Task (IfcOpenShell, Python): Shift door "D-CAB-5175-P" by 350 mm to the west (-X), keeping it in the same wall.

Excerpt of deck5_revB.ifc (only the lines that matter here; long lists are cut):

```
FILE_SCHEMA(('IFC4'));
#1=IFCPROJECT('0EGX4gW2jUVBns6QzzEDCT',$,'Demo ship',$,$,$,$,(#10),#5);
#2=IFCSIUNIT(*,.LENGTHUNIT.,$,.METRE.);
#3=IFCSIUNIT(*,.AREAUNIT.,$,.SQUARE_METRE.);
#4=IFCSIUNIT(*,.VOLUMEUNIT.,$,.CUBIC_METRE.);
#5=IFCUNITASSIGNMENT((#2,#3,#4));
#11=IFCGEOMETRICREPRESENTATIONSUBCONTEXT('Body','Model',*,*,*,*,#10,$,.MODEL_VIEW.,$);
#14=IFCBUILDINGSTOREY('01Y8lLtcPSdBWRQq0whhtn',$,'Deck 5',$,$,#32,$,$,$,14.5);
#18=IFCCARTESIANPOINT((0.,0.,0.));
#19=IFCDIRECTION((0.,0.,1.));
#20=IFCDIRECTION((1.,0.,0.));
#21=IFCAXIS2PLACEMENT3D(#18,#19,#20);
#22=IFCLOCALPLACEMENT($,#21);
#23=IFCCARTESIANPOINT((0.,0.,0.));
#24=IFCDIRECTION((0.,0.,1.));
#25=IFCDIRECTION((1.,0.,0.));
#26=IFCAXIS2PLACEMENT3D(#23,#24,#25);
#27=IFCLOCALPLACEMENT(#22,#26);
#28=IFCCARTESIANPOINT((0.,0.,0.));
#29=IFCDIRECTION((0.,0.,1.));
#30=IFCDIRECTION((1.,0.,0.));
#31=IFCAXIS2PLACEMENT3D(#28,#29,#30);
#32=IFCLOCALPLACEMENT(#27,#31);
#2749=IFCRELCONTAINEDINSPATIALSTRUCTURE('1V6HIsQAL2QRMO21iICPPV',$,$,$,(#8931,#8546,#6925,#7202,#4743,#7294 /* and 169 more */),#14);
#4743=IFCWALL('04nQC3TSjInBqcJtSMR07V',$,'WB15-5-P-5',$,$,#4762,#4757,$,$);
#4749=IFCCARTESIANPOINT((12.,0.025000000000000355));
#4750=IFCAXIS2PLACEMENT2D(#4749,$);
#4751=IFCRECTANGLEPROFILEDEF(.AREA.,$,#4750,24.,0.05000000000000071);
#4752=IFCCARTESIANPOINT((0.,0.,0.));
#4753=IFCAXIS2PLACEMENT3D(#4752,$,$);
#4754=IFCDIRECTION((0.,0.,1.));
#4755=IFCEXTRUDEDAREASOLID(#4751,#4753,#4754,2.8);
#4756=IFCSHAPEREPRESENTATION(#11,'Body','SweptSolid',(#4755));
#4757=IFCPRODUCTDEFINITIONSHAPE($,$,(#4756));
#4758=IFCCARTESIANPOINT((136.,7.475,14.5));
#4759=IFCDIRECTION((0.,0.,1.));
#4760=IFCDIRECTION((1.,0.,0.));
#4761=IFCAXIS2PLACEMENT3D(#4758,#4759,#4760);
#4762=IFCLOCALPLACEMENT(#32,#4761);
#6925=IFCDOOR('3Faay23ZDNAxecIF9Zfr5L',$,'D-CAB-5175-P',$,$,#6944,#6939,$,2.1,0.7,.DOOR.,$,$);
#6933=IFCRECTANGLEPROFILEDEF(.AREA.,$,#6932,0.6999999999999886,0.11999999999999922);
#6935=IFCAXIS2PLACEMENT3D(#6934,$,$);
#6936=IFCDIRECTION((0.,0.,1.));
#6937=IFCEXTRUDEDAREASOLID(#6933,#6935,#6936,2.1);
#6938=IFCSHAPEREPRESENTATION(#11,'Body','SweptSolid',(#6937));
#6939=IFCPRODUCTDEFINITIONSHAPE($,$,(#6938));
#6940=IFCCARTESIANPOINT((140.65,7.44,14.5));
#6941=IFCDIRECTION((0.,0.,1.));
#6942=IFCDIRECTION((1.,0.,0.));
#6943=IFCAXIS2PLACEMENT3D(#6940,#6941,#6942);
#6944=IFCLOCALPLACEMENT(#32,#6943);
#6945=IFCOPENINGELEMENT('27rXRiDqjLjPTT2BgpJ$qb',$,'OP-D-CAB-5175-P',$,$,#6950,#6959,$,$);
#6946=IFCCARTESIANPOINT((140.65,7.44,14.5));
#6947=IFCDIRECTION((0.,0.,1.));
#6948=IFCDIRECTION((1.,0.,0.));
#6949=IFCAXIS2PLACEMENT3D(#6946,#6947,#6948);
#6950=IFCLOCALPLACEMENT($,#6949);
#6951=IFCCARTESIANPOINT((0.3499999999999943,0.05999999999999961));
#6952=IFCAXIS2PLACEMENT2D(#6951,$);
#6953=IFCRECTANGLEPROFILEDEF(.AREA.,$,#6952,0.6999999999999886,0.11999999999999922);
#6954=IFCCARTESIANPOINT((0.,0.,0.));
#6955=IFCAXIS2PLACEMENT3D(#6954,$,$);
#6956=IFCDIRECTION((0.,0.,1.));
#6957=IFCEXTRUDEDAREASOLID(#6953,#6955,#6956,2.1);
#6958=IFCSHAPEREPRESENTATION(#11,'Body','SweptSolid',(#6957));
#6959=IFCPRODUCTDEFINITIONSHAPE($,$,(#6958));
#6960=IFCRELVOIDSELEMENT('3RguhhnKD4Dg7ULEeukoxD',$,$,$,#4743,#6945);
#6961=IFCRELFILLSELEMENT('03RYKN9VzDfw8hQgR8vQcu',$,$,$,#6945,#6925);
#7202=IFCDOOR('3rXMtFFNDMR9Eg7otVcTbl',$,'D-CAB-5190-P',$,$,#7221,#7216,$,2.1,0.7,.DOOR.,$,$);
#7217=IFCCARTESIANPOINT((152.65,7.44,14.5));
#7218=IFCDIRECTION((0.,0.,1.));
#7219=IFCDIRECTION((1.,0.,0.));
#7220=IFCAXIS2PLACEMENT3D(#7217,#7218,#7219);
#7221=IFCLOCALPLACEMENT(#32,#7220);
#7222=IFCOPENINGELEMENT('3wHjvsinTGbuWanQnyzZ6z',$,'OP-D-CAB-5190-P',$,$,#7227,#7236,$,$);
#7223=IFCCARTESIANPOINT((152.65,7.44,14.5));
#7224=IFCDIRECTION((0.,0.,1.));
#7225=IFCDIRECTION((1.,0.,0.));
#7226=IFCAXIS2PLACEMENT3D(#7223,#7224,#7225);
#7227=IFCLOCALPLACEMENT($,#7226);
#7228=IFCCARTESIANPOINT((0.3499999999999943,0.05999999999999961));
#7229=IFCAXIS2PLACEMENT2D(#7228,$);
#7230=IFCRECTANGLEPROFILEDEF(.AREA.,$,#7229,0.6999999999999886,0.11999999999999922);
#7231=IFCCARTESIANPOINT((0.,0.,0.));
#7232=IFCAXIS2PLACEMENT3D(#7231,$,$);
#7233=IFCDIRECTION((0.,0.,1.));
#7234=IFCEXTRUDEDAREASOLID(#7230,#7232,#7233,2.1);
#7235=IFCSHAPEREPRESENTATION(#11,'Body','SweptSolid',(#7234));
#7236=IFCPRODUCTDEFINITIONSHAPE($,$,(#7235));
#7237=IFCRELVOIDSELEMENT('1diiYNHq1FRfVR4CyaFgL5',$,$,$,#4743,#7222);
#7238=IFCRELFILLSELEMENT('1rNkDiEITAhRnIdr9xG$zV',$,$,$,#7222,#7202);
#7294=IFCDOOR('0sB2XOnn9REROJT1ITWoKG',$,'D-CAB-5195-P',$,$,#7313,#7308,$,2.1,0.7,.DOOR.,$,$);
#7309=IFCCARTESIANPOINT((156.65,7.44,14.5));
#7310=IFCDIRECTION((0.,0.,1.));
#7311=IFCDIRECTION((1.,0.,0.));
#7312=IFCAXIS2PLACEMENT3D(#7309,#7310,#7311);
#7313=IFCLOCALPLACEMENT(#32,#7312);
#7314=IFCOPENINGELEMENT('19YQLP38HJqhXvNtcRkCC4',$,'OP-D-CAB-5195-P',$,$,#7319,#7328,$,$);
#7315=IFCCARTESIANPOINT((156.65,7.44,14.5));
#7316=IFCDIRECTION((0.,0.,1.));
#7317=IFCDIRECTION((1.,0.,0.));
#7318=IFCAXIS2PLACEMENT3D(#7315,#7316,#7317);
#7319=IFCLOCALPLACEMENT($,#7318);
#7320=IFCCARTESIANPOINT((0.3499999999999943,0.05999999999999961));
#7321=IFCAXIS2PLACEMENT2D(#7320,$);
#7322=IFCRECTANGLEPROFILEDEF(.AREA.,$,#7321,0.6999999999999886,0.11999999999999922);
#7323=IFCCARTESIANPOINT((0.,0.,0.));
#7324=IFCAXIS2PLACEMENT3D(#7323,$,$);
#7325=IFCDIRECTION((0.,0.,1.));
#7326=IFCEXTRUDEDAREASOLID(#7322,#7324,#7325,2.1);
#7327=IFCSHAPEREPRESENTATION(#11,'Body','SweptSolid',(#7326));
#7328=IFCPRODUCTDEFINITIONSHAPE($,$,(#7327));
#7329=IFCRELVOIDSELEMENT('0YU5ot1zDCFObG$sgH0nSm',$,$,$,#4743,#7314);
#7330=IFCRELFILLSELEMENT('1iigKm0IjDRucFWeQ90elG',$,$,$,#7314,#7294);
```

```python
import ifcopenshell
import ifcopenshell.api.geometry
import ifcopenshell.util.placement
import ifcopenshell.util.unit

model = ifcopenshell.open("deck5_revB.ifc")
unit_scale = ifcopenshell.util.unit.calculate_unit_scale(model)

door = model.by_id(6925)
opening = door.FillsVoids[0].RelatingOpeningElement
wall = opening.VoidsElements[0].RelatingBuildingElement

wall_matrix = ifcopenshell.util.placement.get_local_placement(wall.ObjectPlacement)
shift = wall_matrix[:3, 0] * -0.35 / unit_scale
before = ifcopenshell.util.placement.get_local_placement(door.ObjectPlacement)[:3, 3].copy()

# The door is not placed relative to its opening, so move both.
for product in (opening, door):
    matrix = ifcopenshell.util.placement.get_local_placement(product.ObjectPlacement)
    matrix[:3, 3] += shift
    ifcopenshell.api.geometry.edit_object_placement(model, product=product, matrix=matrix, is_si=False)

after = ifcopenshell.util.placement.get_local_placement(door.ObjectPlacement)[:3, 3]
print("door moved by", (after - before).round(3) + 0.0)

model.write("deck5_revB_updated.ifc")
```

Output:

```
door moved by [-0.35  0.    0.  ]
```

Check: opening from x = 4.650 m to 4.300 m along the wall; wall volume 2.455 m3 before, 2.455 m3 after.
